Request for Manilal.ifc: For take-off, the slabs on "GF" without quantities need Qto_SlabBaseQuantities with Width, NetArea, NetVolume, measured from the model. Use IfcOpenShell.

First a look at what the model holds.

```python
import ifcopenshell
import ifcopenshell.util.element
import ifcopenshell.util.unit

model = ifcopenshell.open("Manilal.ifc")
print(model.schema)
for unit_type in ("LENGTHUNIT", "AREAUNIT", "VOLUMEUNIT"):
    print(unit_type, ifcopenshell.util.unit.calculate_unit_scale(model, unit_type))
storey = next(s for s in model.by_type("IfcBuildingStorey") if s.Name == "GF")
slabs = [e for e in ifcopenshell.util.element.get_decomposition(storey) if e.is_a("IfcSlab")]
for e in sorted(slabs, key=lambda e: e.id()):
    print(e.id(), e.is_a(), e.Name, list(ifcopenshell.util.element.get_psets(e, qtos_only=True)), sep=" | ")
```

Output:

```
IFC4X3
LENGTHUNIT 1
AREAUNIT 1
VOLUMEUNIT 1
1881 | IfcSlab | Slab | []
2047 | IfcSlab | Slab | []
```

```python
import ifcopenshell
import ifcopenshell.api.pset
import ifcopenshell.geom
import ifcopenshell.util.element
import ifcopenshell.util.shape
import ifcopenshell.util.unit

model = ifcopenshell.open("Manilal.ifc")
unit_scale = ifcopenshell.util.unit.calculate_unit_scale(model)
area_scale = ifcopenshell.util.unit.calculate_unit_scale(model, "AREAUNIT")
volume_scale = ifcopenshell.util.unit.calculate_unit_scale(model, "VOLUMEUNIT")
settings = ifcopenshell.geom.settings()

storey = next(s for s in model.by_type("IfcBuildingStorey") if s.Name == "GF")
slabs = [e for e in ifcopenshell.util.element.get_decomposition(storey) if e.is_a("IfcSlab")]

for e in sorted(slabs, key=lambda e: e.id()):
    if ifcopenshell.util.element.get_psets(e, qtos_only=True, should_inherit=False):
        continue
    # Geometry comes back in metres, in the element's own axes.
    shape = ifcopenshell.geom.create_shape(settings, e)
    values = {
        "Width": ifcopenshell.util.shape.get_z(shape.geometry) / unit_scale,
        "NetArea": ifcopenshell.util.shape.get_footprint_area(shape.geometry) / area_scale,
        "NetVolume": ifcopenshell.util.shape.get_volume(shape.geometry) / volume_scale,
    }
    qto = ifcopenshell.api.pset.add_qto(model, product=e, name="Qto_SlabBaseQuantities")
    ifcopenshell.api.pset.edit_qto(model, qto=qto, properties=values)
    print(e.id(), {k: round(v, 3) for k, v in values.items()})

model.write("Manilal_updated.ifc")
```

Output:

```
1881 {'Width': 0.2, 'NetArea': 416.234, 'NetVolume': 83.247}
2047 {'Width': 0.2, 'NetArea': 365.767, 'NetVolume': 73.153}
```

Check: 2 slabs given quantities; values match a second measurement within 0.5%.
